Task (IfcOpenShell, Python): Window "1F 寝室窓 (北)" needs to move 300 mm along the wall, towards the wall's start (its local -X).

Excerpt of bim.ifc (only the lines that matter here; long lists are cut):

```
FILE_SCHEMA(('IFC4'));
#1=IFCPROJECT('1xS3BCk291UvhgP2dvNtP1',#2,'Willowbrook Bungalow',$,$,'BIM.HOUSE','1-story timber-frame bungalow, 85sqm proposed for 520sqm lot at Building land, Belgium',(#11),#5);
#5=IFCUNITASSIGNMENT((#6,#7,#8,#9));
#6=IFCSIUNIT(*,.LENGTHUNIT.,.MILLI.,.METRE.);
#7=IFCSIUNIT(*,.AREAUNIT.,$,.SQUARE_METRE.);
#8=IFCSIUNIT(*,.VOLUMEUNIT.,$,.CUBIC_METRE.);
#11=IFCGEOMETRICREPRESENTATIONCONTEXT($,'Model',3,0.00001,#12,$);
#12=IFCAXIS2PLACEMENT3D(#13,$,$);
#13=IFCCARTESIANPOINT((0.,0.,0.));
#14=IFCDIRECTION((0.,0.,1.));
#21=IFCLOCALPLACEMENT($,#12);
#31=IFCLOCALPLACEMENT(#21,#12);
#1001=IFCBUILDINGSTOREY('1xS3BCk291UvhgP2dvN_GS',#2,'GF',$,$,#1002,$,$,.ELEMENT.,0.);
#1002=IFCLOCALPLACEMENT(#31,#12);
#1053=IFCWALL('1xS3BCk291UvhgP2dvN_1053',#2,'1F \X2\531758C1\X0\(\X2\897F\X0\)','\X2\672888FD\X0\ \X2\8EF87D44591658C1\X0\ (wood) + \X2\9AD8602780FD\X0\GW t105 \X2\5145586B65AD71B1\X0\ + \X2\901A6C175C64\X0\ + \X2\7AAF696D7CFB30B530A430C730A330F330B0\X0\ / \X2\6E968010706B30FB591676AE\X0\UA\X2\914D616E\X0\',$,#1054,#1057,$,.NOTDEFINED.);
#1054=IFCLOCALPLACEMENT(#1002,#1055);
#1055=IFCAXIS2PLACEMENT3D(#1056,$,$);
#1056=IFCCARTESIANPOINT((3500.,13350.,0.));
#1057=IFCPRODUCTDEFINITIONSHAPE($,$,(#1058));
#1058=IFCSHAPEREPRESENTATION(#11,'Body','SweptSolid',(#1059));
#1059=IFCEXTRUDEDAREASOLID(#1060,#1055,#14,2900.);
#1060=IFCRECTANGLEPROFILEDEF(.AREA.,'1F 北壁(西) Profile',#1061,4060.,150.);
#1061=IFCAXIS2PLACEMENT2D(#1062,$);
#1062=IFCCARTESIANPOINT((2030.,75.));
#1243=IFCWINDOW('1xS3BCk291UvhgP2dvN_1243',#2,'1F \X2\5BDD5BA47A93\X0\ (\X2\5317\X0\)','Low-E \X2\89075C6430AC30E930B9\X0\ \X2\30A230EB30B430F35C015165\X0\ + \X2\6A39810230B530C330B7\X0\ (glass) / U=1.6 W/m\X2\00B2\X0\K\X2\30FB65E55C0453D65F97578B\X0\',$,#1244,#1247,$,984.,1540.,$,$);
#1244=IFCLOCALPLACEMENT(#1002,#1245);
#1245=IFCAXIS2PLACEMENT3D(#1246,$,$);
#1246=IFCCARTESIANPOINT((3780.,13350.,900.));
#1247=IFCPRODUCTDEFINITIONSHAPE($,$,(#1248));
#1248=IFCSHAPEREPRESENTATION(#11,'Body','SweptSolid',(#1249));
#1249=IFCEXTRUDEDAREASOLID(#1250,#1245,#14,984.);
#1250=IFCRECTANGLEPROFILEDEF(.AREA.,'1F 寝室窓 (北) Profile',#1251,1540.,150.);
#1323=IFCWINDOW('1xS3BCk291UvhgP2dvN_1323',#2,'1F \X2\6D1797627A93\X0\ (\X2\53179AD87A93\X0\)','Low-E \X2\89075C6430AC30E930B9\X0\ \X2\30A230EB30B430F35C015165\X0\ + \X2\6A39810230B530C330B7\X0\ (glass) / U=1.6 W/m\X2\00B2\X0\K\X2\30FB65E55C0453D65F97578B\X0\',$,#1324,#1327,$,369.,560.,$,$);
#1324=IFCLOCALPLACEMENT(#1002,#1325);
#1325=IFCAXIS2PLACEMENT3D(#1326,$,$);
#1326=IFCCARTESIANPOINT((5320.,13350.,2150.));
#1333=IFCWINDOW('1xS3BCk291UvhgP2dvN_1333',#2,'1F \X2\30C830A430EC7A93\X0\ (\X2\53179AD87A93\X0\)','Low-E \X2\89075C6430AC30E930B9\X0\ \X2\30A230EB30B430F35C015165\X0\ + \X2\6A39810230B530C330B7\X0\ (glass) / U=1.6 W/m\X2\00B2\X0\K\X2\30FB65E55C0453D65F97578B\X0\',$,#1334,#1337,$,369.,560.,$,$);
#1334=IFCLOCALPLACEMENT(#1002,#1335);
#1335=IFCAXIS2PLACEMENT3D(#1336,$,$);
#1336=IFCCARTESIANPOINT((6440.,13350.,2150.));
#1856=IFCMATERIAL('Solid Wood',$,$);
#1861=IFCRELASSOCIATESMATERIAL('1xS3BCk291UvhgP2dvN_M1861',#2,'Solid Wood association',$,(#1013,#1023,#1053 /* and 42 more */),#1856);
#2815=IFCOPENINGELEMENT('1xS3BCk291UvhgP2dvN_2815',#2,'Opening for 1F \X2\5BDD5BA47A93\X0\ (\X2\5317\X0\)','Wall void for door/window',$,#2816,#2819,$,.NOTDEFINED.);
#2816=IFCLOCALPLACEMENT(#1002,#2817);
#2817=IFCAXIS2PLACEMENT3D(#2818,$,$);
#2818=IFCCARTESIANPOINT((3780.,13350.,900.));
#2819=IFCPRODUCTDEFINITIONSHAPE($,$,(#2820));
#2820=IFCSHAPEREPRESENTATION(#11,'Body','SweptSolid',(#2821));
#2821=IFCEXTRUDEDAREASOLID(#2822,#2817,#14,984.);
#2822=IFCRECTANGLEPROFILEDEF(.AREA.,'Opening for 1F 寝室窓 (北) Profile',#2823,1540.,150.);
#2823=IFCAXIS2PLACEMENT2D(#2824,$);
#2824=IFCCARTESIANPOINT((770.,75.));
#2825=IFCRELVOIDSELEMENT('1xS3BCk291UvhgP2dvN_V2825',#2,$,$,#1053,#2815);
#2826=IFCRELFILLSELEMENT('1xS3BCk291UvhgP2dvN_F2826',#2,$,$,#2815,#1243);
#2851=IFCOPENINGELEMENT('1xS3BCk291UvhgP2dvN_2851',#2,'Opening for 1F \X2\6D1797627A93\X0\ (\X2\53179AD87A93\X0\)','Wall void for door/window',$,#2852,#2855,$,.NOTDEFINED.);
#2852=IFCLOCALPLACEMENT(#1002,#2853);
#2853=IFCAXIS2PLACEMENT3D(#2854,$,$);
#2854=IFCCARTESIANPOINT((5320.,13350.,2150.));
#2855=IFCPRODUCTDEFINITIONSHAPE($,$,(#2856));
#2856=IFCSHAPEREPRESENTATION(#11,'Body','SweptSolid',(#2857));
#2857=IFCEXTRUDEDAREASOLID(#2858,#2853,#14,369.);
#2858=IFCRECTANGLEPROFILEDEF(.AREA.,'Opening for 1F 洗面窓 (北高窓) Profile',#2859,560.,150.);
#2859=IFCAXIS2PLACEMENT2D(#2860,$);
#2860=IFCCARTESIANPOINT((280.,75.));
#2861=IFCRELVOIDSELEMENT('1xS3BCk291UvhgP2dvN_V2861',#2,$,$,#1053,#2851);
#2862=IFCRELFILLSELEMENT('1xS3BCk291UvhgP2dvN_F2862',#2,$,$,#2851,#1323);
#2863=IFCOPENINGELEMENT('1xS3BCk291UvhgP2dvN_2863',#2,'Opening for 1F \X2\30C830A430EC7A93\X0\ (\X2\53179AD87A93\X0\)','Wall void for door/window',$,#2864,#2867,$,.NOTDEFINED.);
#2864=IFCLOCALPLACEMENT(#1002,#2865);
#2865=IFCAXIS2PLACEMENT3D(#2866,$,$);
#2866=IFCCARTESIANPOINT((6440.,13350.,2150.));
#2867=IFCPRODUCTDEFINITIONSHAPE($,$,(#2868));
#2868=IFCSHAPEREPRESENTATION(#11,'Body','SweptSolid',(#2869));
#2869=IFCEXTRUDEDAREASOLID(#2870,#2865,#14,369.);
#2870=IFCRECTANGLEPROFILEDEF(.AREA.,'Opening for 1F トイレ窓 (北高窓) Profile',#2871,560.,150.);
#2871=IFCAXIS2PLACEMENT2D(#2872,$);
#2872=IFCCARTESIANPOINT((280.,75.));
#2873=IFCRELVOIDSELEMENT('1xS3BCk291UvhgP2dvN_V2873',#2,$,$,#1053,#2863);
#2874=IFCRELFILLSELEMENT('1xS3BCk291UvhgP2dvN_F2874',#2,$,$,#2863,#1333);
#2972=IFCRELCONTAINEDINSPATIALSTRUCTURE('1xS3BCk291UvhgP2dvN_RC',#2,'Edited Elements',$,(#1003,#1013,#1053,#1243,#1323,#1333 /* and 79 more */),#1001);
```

```python
import ifcopenshell
import ifcopenshell.api.geometry
import ifcopenshell.util.placement

model = ifcopenshell.open("bim.ifc")

window = model.by_guid("1xS3BCk291UvhgP2dvN_1243")
opening = window.FillsVoids[0].RelatingOpeningElement
wall = opening.VoidsElements[0].RelatingBuildingElement

wall_matrix = ifcopenshell.util.placement.get_local_placement(wall.ObjectPlacement)
shift = wall_matrix[:3, 0] * -300.0
before = ifcopenshell.util.placement.get_local_placement(window.ObjectPlacement)[:3, 3].copy()

# The window is not placed relative to its opening, so move both.
for product in (opening, window):
    matrix = ifcopenshell.util.placement.get_local_placement(product.ObjectPlacement)
    matrix[:3, 3] += shift
    ifcopenshell.api.geometry.edit_object_placement(model, product=product, matrix=matrix, is_si=False)

after = ifcopenshell.util.placement.get_local_placement(window.ObjectPlacement)[:3, 3]
print("window moved by", (after - before).round(3) + 0.0)

model.write("bim_v2.ifc")
```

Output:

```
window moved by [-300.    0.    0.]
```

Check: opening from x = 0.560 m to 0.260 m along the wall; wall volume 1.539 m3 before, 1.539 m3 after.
